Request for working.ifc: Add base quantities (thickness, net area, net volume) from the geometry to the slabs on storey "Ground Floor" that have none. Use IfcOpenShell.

First a look at what the model holds.

```python
import ifcopenshell
import ifcopenshell.util.element
import ifcopenshell.util.unit

model = ifcopenshell.open("working.ifc")
print(model.schema)
for unit_type in ("LENGTHUNIT", "AREAUNIT", "VOLUMEUNIT"):
    print(unit_type, ifcopenshell.util.unit.calculate_unit_scale(model, unit_type))
storey = next(s for s in model.by_type("IfcBuildingStorey") if s.Name == "Ground Floor")
slabs = [e for e in ifcopenshell.util.element.get_decomposition(storey) if e.is_a("IfcSlab")]
for e in sorted(slabs, key=lambda e: e.id()):
    print(e.id(), e.is_a(), e.Name, list(ifcopenshell.util.element.get_psets(e, qtos_only=True)), sep=" | ")
```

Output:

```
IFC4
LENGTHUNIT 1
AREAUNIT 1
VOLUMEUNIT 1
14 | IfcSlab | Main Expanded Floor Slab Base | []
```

```python
import ifcopenshell
import ifcopenshell.api.pset
import ifcopenshell.geom
import ifcopenshell.util.element
import ifcopenshell.util.shape
import ifcopenshell.util.unit

model = ifcopenshell.open("working.ifc")
unit_scale = ifcopenshell.util.unit.calculate_unit_scale(model)
area_scale = ifcopenshell.util.unit.calculate_unit_scale(model, "AREAUNIT")
volume_scale = ifcopenshell.util.unit.calculate_unit_scale(model, "VOLUMEUNIT")
settings = ifcopenshell.geom.settings()

storey = next(s for s in model.by_type("IfcBuildingStorey") if s.Name == "Ground Floor")
slabs = [e for e in ifcopenshell.util.element.get_decomposition(storey) if e.is_a("IfcSlab")]

for e in sorted(slabs, key=lambda e: e.id()):
    if ifcopenshell.util.element.get_psets(e, qtos_only=True, should_inherit=False):
        continue
    # Geometry comes back in metres, in the element's own axes.
    shape = ifcopenshell.geom.create_shape(settings, e)
    values = {
        "Width": ifcopenshell.util.shape.get_z(shape.geometry) / unit_scale,
        "NetArea": ifcopenshell.util.shape.get_footprint_area(shape.geometry) / area_scale,
        "NetVolume": ifcopenshell.util.shape.get_volume(shape.geometry) / volume_scale,
    }
    qto = ifcopenshell.api.pset.add_qto(model, product=e, name="Qto_SlabBaseQuantities")
    ifcopenshell.api.pset.edit_qto(model, qto=qto, properties=values)
    print(e.id(), {k: round(v, 3) for k, v in values.items()})

model.write("working_edited.ifc")
```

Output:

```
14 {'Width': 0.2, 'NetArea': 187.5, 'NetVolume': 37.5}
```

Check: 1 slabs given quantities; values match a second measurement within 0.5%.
